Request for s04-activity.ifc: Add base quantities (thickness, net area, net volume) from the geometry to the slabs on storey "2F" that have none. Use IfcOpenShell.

First a look at what the model holds.

```python
import ifcopenshell
import ifcopenshell.util.element
import ifcopenshell.util.unit

model = ifcopenshell.open("s04-activity.ifc")
print(model.schema)
for unit_type in ("LENGTHUNIT", "AREAUNIT", "VOLUMEUNIT"):
    print(unit_type, ifcopenshell.util.unit.calculate_unit_scale(model, unit_type))
storey = next(s for s in model.by_type("IfcBuildingStorey") if s.Name == "2F")
slabs = [e for e in ifcopenshell.util.element.get_decomposition(storey) if e.is_a("IfcSlab")]
for e in sorted(slabs, key=lambda e: e.id()):
    print(e.id(), e.is_a(), e.Name, list(ifcopenshell.util.element.get_psets(e, qtos_only=True)), sep=" | ")
```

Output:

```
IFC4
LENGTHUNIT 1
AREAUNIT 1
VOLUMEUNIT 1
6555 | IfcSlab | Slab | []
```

```python
import ifcopenshell
import ifcopenshell.api.pset
import ifcopenshell.geom
import ifcopenshell.util.element
import ifcopenshell.util.shape
import ifcopenshell.util.unit

model = ifcopenshell.open("s04-activity.ifc")
unit_scale = ifcopenshell.util.unit.calculate_unit_scale(model)
area_scale = ifcopenshell.util.unit.calculate_unit_scale(model, "AREAUNIT")
volume_scale = ifcopenshell.util.unit.calculate_unit_scale(model, "VOLUMEUNIT")
settings = ifcopenshell.geom.settings()

storey = next(s for s in model.by_type("IfcBuildingStorey") if s.Name == "2F")
slabs = [e for e in ifcopenshell.util.element.get_decomposition(storey) if e.is_a("IfcSlab")]

for e in sorted(slabs, key=lambda e: e.id()):
    if ifcopenshell.util.element.get_psets(e, qtos_only=True, should_inherit=False):
        continue
    # Geometry comes back in metres, in the element's own axes.
    shape = ifcopenshell.geom.create_shape(settings, e)
    values = {
        "Width": ifcopenshell.util.shape.get_z(shape.geometry) / unit_scale,
        "NetArea": ifcopenshell.util.shape.get_footprint_area(shape.geometry) / area_scale,
        "NetVolume": ifcopenshell.util.shape.get_volume(shape.geometry) / volume_scale,
    }
    qto = ifcopenshell.api.pset.add_qto(model, product=e, name="Qto_SlabBaseQuantities")
    ifcopenshell.api.pset.edit_qto(model, qto=qto, properties=values)
    print(e.id(), {k: round(v, 3) for k, v in values.items()})

model.write("s04-activity_edited.ifc")
```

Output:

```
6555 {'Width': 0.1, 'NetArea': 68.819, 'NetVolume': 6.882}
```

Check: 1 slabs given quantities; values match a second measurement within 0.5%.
